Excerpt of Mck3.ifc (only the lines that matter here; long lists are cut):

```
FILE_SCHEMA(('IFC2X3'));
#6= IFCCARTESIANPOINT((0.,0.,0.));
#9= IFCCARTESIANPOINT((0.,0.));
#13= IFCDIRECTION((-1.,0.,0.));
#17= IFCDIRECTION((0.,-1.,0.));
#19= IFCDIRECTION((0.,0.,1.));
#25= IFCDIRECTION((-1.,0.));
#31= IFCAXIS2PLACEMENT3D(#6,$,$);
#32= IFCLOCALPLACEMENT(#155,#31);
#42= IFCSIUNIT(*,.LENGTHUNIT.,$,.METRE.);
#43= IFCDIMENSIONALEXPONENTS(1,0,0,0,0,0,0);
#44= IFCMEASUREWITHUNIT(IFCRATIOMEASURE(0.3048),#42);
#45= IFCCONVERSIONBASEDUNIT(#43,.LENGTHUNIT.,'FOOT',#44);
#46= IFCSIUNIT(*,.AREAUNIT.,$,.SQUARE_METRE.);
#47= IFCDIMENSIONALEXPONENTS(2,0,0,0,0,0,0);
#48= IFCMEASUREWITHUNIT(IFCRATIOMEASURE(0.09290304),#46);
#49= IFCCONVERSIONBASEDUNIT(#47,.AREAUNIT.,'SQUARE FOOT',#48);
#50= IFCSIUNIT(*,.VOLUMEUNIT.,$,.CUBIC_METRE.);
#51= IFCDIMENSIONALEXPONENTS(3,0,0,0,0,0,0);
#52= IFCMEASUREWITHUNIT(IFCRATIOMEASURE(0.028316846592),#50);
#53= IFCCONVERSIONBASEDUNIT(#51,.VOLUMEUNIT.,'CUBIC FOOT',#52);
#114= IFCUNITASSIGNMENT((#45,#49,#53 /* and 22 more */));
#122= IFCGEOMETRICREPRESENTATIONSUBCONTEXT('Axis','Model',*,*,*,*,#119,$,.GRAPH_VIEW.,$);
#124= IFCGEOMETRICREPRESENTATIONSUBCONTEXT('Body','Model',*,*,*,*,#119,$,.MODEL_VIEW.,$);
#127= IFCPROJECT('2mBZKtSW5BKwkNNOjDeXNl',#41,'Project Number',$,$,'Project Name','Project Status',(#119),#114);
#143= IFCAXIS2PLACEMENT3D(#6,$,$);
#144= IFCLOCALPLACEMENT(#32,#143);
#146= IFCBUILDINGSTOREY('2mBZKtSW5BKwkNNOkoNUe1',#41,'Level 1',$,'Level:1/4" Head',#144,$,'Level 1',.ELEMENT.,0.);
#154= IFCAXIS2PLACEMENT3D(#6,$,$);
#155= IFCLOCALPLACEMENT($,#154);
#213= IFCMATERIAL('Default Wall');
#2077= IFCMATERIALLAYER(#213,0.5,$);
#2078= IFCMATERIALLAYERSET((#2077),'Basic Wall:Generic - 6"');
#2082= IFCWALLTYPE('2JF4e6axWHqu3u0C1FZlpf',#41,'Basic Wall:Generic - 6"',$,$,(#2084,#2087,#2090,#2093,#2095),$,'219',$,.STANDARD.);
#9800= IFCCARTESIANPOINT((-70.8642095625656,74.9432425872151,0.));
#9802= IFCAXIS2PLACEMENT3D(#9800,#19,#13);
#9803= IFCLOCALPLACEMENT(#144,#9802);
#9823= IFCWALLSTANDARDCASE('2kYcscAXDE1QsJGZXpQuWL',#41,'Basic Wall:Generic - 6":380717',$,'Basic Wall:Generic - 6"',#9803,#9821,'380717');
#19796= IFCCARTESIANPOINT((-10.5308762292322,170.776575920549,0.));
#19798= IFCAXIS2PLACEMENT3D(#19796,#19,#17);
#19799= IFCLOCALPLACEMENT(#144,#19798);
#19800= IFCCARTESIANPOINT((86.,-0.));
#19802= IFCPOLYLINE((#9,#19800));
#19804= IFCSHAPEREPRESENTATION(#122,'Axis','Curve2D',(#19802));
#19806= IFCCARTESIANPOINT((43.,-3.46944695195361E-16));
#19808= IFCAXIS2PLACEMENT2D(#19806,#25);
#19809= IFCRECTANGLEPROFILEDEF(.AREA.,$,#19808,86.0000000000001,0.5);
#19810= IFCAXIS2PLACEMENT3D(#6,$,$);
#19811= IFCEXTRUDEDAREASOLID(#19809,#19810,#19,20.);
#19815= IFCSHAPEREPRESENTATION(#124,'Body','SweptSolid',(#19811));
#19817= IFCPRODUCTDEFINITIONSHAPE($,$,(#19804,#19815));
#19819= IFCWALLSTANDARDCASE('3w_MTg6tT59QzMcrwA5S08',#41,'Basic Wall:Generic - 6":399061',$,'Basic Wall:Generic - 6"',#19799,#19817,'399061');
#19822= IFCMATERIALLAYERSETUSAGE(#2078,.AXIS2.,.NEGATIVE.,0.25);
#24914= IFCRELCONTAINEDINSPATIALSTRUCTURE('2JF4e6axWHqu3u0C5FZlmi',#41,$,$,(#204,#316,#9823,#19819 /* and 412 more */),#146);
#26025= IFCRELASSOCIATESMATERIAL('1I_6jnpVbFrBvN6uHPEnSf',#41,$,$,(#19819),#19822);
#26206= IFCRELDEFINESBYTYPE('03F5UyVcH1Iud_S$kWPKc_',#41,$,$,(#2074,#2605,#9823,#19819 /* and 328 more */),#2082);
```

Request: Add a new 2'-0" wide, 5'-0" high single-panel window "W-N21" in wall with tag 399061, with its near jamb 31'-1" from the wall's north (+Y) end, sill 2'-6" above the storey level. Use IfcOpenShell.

```python
import numpy as np
import ifcopenshell
import ifcopenshell.api.feature
import ifcopenshell.api.geometry
import ifcopenshell.api.root
import ifcopenshell.api.spatial
import ifcopenshell.api.type
import ifcopenshell.geom
import ifcopenshell.util.element
import ifcopenshell.util.placement
import ifcopenshell.util.representation
import ifcopenshell.util.shape
import ifcopenshell.util.unit

model = ifcopenshell.open("Mck3.ifc")
unit_scale = ifcopenshell.util.unit.calculate_unit_scale(model)
settings = ifcopenshell.geom.settings()


def volume(element):
    """Net volume in cubic metres, openings subtracted."""
    shape = ifcopenshell.geom.create_shape(settings, element)
    return ifcopenshell.util.shape.get_volume(shape.geometry)


wall = model.by_guid("3w_MTg6tT59QzMcrwA5S08")
storey = ifcopenshell.util.element.get_container(wall, ifc_class="IfcBuildingStorey")
context = ifcopenshell.util.representation.get_context(model, "Model", "Body", "MODEL_VIEW")
before = volume(wall)

width, height, from_end, sill = 0.6096, 1.524, 9.4742, 0.762  # metres

# The wall runs along its own X axis, and the end named is its -X end.
wall_shape = ifcopenshell.geom.create_shape(settings, wall)
x, y, z = ifcopenshell.util.shape.get_vertices(wall_shape.geometry).T
start = x.min() + from_end
face, thickness = float(y.min()), float(y.max() - y.min())
wall_matrix = ifcopenshell.util.placement.get_local_placement(wall.ObjectPlacement)
level = ifcopenshell.util.placement.get_local_placement(storey.ObjectPlacement)[2, 3]


def in_wall(x, y):
    """Placement at x, y metres in the wall's axes, at sill height."""
    matrix = wall_matrix.copy()
    matrix[:, 3] = wall_matrix @ np.array([x / unit_scale, y / unit_scale, 0.0, 1.0])
    matrix[2, 3] = level + sill / unit_scale
    return matrix


# Opening: a box that overshoots both wall faces by 50 mm.
opening = ifcopenshell.api.root.create_entity(model, ifc_class="IfcOpeningElement")
box = ifcopenshell.api.geometry.add_wall_representation(
    model, context=context, length=width, height=height, thickness=thickness + 0.1
)
ifcopenshell.api.geometry.assign_representation(model, product=opening, representation=box)
ifcopenshell.api.geometry.edit_object_placement(model, product=opening, matrix=in_wall(start, face - 0.05), is_si=False)
ifcopenshell.api.feature.add_feature(model, feature=opening, element=wall)

window = ifcopenshell.api.root.create_entity(model, ifc_class="IfcWindow", name="W-N21")
window.OverallWidth, window.OverallHeight = width / unit_scale, height / unit_scale
body = ifcopenshell.api.geometry.add_window_representation(
    model,
    context=context,
    overall_width=window.OverallWidth,
    overall_height=window.OverallHeight,
    partition_type="SINGLE_PANEL",
)
ifcopenshell.api.geometry.assign_representation(model, product=window, representation=body)
ifcopenshell.api.spatial.assign_container(model, products=[window], relating_structure=storey)
fills = ifcopenshell.api.feature.add_filling(model, opening=opening, element=window)
fills.OwnerHistory = window.OwnerHistory  # required in IFC2X3

# IFC2X3 keeps the operation on the window style.
style = ifcopenshell.api.root.create_entity(model, ifc_class="IfcWindowStyle", name="W-N21")
style.OperationType, style.ConstructionType = "SINGLE_PANEL", "NOTDEFINED"
style.ParameterTakesPrecedence = style.Sizeable = False
ifcopenshell.api.type.assign_type(model, related_objects=[window], relating_type=style)

# Centre the window in the wall's thickness.
ifcopenshell.api.geometry.edit_object_placement(model, product=window, matrix=in_wall(start, face), is_si=False)
window_shape = ifcopenshell.geom.create_shape(settings, window)
depth = ifcopenshell.util.shape.get_vertices(window_shape.geometry)[:, 1]
offset = face + thickness / 2 - (depth.min() + depth.max()) / 2
ifcopenshell.api.geometry.edit_object_placement(model, product=window, matrix=in_wall(start, offset), is_si=False)

after = volume(wall)

print(f"wall volume {before:.3f} -> {after:.3f} m3")

model.write("Mck3_edited.ifc")
```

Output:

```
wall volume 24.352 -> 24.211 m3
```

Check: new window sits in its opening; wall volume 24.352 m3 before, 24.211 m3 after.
